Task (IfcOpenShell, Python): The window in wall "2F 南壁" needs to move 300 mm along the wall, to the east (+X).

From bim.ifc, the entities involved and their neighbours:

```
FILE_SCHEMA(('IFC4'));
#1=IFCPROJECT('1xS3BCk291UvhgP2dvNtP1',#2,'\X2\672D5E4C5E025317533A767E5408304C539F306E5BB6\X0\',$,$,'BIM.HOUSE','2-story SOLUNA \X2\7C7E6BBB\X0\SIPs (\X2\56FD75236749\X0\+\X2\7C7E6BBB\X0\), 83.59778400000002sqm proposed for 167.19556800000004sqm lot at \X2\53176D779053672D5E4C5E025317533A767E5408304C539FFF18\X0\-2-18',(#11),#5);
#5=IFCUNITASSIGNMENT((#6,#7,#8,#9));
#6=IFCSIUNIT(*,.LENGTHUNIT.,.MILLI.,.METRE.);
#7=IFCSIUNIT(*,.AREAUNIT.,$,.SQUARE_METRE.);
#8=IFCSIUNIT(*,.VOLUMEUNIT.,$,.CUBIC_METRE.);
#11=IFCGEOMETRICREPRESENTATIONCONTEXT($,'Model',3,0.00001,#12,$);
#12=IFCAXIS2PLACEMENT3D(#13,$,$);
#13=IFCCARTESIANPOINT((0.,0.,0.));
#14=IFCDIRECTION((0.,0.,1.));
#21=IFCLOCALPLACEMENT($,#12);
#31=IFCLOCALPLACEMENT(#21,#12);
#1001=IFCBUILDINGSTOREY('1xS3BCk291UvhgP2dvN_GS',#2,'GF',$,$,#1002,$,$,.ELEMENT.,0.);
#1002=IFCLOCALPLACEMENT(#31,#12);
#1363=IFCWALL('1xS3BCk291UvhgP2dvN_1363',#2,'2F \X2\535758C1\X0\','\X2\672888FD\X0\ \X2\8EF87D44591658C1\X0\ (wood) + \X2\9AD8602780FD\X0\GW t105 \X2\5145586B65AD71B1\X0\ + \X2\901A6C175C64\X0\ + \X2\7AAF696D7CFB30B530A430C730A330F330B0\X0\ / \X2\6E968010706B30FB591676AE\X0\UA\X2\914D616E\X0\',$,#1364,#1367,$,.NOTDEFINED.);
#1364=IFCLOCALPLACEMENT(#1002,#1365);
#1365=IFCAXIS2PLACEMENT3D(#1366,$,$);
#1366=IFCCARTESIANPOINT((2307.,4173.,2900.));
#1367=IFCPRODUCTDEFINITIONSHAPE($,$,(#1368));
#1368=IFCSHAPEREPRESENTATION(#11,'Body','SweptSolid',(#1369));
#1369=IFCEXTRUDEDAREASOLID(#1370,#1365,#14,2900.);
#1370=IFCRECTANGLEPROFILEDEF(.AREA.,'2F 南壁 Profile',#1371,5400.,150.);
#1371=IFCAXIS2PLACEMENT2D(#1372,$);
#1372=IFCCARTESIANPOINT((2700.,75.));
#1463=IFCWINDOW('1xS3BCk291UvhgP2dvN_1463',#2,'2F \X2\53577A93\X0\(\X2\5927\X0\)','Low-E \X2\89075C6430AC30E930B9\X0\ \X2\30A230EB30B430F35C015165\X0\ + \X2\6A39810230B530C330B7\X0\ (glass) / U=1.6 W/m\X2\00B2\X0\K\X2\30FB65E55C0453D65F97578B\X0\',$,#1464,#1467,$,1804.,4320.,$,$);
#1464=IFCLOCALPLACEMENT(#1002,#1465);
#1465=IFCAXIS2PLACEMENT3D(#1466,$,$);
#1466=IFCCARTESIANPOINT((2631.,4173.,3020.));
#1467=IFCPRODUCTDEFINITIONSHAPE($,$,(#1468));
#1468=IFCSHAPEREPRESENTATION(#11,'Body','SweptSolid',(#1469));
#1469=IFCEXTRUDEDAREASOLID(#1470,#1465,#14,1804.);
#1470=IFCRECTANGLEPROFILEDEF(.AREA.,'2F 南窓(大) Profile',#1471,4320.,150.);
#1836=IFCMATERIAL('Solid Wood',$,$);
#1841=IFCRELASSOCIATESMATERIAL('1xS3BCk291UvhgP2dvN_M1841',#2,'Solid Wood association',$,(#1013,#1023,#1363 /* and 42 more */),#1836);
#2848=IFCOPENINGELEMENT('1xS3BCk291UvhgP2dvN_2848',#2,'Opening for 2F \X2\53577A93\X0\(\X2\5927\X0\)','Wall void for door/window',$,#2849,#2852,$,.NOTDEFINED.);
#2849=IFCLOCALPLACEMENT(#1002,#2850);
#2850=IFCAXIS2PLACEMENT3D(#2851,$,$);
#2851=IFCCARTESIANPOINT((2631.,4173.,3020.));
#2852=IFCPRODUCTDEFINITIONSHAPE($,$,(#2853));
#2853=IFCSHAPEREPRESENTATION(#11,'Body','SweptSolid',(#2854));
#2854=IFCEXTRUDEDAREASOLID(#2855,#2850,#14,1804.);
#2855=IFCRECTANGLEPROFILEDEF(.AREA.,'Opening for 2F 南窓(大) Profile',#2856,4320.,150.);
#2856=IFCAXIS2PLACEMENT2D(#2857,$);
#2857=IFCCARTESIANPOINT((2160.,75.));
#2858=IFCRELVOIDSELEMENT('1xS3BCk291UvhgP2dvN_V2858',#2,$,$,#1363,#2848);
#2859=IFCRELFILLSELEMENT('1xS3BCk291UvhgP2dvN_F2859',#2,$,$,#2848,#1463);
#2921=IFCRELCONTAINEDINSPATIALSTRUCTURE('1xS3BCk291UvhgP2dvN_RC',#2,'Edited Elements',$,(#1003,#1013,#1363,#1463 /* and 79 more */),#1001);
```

```python
import ifcopenshell
import ifcopenshell.api.geometry
import ifcopenshell.util.placement

model = ifcopenshell.open("bim.ifc")

window = model.by_id(1463)
opening = window.FillsVoids[0].RelatingOpeningElement
wall = opening.VoidsElements[0].RelatingBuildingElement

wall_matrix = ifcopenshell.util.placement.get_local_placement(wall.ObjectPlacement)
shift = wall_matrix[:3, 0] * 300.0
before = ifcopenshell.util.placement.get_local_placement(window.ObjectPlacement)[:3, 3].copy()

# The window is not placed relative to its opening, so move both.
for product in (opening, window):
    matrix = ifcopenshell.util.placement.get_local_placement(product.ObjectPlacement)
    matrix[:3, 3] += shift
    ifcopenshell.api.geometry.edit_object_placement(model, product=product, matrix=matrix, is_si=False)

after = ifcopenshell.util.placement.get_local_placement(window.ObjectPlacement)[:3, 3]
print("window moved by", (after - before).round(3) + 0.0)

model.write("bim-out.ifc")
```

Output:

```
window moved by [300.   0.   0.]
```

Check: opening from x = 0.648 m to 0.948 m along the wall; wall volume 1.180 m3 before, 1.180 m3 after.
